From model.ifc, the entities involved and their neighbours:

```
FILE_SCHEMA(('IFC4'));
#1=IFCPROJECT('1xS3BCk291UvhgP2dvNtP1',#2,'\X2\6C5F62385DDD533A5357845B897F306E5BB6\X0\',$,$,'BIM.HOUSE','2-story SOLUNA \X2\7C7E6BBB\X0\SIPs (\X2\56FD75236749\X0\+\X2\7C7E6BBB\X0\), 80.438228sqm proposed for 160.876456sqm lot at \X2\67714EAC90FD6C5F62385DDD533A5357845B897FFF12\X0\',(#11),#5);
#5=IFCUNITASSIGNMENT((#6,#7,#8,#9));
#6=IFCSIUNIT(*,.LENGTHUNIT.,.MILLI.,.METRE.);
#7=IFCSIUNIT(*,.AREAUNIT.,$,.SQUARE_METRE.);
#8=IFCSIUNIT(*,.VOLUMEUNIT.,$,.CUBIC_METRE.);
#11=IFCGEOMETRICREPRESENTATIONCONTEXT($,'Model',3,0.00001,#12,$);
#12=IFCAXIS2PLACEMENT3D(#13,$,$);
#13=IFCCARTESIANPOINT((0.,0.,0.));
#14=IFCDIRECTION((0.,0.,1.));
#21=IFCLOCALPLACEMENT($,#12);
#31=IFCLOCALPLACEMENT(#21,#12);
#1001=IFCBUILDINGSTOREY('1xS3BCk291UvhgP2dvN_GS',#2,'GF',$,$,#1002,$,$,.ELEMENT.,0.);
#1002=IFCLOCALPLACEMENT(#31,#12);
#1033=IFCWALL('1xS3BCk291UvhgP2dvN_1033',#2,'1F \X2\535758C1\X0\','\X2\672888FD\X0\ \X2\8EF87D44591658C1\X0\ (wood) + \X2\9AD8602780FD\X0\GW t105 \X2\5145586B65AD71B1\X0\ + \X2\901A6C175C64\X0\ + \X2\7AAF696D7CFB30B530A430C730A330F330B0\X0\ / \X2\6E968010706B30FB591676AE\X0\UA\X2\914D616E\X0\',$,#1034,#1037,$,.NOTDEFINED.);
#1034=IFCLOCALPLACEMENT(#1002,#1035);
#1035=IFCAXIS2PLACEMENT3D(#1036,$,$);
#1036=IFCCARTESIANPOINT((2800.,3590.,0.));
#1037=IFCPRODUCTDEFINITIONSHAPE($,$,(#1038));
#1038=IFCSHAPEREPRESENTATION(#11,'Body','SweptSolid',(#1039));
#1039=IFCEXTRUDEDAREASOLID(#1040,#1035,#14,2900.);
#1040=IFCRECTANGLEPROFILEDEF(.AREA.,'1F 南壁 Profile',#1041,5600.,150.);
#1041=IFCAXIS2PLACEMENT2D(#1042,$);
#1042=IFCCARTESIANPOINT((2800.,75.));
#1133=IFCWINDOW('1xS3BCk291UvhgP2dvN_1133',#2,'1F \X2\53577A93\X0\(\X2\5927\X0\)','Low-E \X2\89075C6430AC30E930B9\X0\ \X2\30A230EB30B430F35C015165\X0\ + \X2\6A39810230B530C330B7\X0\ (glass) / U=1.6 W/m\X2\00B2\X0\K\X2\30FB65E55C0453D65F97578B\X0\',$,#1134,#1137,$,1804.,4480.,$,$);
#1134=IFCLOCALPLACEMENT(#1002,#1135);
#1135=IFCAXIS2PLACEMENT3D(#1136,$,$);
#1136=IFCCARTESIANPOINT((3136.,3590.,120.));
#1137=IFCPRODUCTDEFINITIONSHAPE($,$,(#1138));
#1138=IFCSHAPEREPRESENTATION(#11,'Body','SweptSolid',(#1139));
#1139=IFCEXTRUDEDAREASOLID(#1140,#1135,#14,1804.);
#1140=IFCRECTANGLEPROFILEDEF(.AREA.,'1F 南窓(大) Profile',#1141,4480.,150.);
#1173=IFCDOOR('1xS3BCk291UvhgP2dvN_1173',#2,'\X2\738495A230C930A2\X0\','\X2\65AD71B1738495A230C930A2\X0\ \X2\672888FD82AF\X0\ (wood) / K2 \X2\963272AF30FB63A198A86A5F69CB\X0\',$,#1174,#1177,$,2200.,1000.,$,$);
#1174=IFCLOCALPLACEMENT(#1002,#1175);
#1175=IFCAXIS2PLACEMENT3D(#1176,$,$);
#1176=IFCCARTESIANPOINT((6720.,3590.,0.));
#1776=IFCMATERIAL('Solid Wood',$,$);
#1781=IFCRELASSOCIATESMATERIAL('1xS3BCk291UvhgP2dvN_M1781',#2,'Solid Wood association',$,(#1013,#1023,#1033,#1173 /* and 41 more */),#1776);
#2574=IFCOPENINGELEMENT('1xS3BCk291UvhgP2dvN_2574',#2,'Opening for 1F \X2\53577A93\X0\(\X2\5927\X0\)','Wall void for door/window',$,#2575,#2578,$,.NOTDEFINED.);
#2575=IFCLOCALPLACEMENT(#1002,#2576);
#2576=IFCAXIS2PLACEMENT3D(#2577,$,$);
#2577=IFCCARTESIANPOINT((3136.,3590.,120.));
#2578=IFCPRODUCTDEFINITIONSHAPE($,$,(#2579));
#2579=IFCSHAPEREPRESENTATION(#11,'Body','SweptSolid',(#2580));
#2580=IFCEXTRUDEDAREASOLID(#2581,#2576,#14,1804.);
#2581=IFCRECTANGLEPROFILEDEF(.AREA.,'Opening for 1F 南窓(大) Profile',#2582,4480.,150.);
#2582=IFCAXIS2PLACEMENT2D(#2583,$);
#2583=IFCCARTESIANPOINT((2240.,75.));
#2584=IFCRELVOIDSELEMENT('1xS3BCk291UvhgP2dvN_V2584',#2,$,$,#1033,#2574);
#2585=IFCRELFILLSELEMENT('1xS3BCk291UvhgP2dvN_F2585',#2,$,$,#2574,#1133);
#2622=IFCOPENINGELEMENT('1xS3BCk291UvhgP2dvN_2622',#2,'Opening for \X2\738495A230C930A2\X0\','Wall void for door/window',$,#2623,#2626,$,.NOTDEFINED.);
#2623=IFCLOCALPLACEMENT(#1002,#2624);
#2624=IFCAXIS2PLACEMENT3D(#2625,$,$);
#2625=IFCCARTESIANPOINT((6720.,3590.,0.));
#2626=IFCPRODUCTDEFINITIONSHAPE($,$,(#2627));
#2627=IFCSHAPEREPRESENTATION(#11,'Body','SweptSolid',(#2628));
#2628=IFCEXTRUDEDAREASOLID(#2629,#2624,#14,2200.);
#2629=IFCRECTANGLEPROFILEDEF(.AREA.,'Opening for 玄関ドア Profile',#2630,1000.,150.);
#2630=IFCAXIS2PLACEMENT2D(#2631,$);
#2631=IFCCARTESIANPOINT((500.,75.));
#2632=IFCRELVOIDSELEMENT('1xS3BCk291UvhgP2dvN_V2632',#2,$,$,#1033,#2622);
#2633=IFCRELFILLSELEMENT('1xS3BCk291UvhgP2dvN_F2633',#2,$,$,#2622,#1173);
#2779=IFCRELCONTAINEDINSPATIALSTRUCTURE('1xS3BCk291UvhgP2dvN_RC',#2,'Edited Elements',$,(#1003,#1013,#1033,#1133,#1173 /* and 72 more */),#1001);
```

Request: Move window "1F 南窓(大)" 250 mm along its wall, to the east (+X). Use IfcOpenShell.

```python
import ifcopenshell
import ifcopenshell.api.geometry
import ifcopenshell.util.placement

model = ifcopenshell.open("model.ifc")

window = model.by_guid("1xS3BCk291UvhgP2dvN_1133")
opening = window.FillsVoids[0].RelatingOpeningElement
wall = opening.VoidsElements[0].RelatingBuildingElement

wall_matrix = ifcopenshell.util.placement.get_local_placement(wall.ObjectPlacement)
shift = wall_matrix[:3, 0] * 250.0
before = ifcopenshell.util.placement.get_local_placement(window.ObjectPlacement)[:3, 3].copy()

# The window is not placed relative to its opening, so move both.
for product in (opening, window):
    matrix = ifcopenshell.util.placement.get_local_placement(product.ObjectPlacement)
    matrix[:3, 3] += shift
    ifcopenshell.api.geometry.edit_object_placement(model, product=product, matrix=matrix, is_si=False)

after = ifcopenshell.util.placement.get_local_placement(window.ObjectPlacement)[:3, 3]
print("window moved by", (after - before).round(3) + 0.0)

model.write("model_updated.ifc")
```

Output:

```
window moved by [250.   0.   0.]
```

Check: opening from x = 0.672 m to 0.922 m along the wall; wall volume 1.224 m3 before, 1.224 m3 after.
